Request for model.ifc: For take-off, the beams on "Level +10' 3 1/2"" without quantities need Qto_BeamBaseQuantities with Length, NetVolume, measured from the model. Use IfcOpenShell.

First a look at what the model holds.

```python
import ifcopenshell
import ifcopenshell.util.element
import ifcopenshell.util.unit

model = ifcopenshell.open("model.ifc")
print(model.schema)
for unit_type in ("LENGTHUNIT", "AREAUNIT", "VOLUMEUNIT"):
    print(unit_type, ifcopenshell.util.unit.calculate_unit_scale(model, unit_type))
storey = next(s for s in model.by_type("IfcBuildingStorey") if s.Name == 'Level +10\' 3 1/2"')
beams = [e for e in ifcopenshell.util.element.get_decomposition(storey) if e.is_a("IfcBeam")]
for e in sorted(beams, key=lambda e: e.id()):
    print(e.id(), e.is_a(), e.Name, list(ifcopenshell.util.element.get_psets(e, qtos_only=True)), sep=" | ")
```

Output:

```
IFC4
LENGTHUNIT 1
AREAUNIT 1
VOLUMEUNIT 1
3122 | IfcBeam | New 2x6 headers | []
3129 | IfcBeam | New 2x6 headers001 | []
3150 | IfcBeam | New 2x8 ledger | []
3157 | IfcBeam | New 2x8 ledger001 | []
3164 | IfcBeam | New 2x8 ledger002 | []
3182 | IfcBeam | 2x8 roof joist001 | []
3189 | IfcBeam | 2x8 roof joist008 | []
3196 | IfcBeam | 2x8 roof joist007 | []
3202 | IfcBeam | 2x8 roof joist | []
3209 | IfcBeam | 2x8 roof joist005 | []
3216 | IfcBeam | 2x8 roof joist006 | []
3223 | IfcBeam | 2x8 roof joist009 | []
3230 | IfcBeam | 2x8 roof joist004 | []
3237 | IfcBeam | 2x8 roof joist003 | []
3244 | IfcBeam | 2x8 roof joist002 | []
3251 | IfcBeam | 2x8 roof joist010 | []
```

```python
import ifcopenshell
import ifcopenshell.api.pset
import ifcopenshell.geom
import ifcopenshell.util.element
import ifcopenshell.util.shape
import ifcopenshell.util.unit

model = ifcopenshell.open("model.ifc")
unit_scale = ifcopenshell.util.unit.calculate_unit_scale(model)
volume_scale = ifcopenshell.util.unit.calculate_unit_scale(model, "VOLUMEUNIT")
settings = ifcopenshell.geom.settings()

storey = next(s for s in model.by_type("IfcBuildingStorey") if s.Name == 'Level +10\' 3 1/2"')
beams = [e for e in ifcopenshell.util.element.get_decomposition(storey) if e.is_a("IfcBeam")]

for e in sorted(beams, key=lambda e: e.id()):
    if ifcopenshell.util.element.get_psets(e, qtos_only=True, should_inherit=False):
        continue
    # Geometry comes back in metres, in the element's own axes.
    shape = ifcopenshell.geom.create_shape(settings, e)
    values = {
        "Length": ifcopenshell.util.shape.get_max_xyz(shape.geometry) / unit_scale,
        "NetVolume": ifcopenshell.util.shape.get_volume(shape.geometry) / volume_scale,
    }
    qto = ifcopenshell.api.pset.add_qto(model, product=e, name="Qto_BeamBaseQuantities")
    ifcopenshell.api.pset.edit_qto(model, qto=qto, properties=values)
    print(e.id(), {k: round(v, 3) for k, v in values.items()})

model.write("model_updated.ifc")
```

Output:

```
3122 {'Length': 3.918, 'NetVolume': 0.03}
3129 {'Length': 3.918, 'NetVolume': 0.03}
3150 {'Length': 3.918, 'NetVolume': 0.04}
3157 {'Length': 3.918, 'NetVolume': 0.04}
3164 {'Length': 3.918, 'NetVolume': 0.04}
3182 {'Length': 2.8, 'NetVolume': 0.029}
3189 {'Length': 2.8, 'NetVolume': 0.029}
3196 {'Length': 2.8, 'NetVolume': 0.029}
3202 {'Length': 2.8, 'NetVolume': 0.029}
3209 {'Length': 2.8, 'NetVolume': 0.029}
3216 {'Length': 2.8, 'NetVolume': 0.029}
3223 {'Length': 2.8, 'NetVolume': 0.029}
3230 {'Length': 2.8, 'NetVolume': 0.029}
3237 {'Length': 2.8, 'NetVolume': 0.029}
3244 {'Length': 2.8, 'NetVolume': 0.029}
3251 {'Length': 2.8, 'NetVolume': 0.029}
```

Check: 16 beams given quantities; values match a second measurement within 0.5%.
